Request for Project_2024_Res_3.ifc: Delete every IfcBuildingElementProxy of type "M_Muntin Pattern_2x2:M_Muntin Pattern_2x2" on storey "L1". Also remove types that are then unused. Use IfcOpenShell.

First a look at what the model holds.

```python
import ifcopenshell
import ifcopenshell.util.element

model = ifcopenshell.open("Project_2024_Res_3.ifc")
print(model.schema)
storey = next(s for s in model.by_type("IfcBuildingStorey") if s.Name == "L1")
proxies = [e for e in ifcopenshell.util.element.get_decomposition(storey) if e.is_a("IfcBuildingElementProxy")]
seen = {}
for e in proxies:
    element_type = ifcopenshell.util.element.get_type(e)
    name = element_type.Name if element_type not in (None, e) else None
    seen[name] = seen.get(name, 0) + 1
for name, count in sorted(seen.items(), key=str):
    print(count, "x", name)
```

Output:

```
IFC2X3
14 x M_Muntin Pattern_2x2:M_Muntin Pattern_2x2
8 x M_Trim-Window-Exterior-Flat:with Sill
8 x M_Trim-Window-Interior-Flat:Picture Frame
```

```python
import ifcopenshell
import ifcopenshell.api.root
import ifcopenshell.util.element

model = ifcopenshell.open("Project_2024_Res_3.ifc")

storey = next(s for s in model.by_type("IfcBuildingStorey") if s.Name == "L1")
proxies = [e for e in ifcopenshell.util.element.get_decomposition(storey) if e.is_a("IfcBuildingElementProxy")]
targets = [e for e in proxies if (t := ifcopenshell.util.element.get_type(e)) not in (None, e) and t.Name == "M_Muntin Pattern_2x2:M_Muntin Pattern_2x2"]
types = {ifcopenshell.util.element.get_type(e) for e in targets} - {None, *targets}

for e in targets:
    ifcopenshell.api.root.remove_product(model, product=e)
print(len(targets), "removed")

unused = [t for t in types if not ifcopenshell.util.element.get_types(t)]
for t in unused:
    ifcopenshell.api.root.remove_product(model, product=t)
print(len(unused), "unused types removed")

model.write("Project_2024_Res_3_updated.ifc")
```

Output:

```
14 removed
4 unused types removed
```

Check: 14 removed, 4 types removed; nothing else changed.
